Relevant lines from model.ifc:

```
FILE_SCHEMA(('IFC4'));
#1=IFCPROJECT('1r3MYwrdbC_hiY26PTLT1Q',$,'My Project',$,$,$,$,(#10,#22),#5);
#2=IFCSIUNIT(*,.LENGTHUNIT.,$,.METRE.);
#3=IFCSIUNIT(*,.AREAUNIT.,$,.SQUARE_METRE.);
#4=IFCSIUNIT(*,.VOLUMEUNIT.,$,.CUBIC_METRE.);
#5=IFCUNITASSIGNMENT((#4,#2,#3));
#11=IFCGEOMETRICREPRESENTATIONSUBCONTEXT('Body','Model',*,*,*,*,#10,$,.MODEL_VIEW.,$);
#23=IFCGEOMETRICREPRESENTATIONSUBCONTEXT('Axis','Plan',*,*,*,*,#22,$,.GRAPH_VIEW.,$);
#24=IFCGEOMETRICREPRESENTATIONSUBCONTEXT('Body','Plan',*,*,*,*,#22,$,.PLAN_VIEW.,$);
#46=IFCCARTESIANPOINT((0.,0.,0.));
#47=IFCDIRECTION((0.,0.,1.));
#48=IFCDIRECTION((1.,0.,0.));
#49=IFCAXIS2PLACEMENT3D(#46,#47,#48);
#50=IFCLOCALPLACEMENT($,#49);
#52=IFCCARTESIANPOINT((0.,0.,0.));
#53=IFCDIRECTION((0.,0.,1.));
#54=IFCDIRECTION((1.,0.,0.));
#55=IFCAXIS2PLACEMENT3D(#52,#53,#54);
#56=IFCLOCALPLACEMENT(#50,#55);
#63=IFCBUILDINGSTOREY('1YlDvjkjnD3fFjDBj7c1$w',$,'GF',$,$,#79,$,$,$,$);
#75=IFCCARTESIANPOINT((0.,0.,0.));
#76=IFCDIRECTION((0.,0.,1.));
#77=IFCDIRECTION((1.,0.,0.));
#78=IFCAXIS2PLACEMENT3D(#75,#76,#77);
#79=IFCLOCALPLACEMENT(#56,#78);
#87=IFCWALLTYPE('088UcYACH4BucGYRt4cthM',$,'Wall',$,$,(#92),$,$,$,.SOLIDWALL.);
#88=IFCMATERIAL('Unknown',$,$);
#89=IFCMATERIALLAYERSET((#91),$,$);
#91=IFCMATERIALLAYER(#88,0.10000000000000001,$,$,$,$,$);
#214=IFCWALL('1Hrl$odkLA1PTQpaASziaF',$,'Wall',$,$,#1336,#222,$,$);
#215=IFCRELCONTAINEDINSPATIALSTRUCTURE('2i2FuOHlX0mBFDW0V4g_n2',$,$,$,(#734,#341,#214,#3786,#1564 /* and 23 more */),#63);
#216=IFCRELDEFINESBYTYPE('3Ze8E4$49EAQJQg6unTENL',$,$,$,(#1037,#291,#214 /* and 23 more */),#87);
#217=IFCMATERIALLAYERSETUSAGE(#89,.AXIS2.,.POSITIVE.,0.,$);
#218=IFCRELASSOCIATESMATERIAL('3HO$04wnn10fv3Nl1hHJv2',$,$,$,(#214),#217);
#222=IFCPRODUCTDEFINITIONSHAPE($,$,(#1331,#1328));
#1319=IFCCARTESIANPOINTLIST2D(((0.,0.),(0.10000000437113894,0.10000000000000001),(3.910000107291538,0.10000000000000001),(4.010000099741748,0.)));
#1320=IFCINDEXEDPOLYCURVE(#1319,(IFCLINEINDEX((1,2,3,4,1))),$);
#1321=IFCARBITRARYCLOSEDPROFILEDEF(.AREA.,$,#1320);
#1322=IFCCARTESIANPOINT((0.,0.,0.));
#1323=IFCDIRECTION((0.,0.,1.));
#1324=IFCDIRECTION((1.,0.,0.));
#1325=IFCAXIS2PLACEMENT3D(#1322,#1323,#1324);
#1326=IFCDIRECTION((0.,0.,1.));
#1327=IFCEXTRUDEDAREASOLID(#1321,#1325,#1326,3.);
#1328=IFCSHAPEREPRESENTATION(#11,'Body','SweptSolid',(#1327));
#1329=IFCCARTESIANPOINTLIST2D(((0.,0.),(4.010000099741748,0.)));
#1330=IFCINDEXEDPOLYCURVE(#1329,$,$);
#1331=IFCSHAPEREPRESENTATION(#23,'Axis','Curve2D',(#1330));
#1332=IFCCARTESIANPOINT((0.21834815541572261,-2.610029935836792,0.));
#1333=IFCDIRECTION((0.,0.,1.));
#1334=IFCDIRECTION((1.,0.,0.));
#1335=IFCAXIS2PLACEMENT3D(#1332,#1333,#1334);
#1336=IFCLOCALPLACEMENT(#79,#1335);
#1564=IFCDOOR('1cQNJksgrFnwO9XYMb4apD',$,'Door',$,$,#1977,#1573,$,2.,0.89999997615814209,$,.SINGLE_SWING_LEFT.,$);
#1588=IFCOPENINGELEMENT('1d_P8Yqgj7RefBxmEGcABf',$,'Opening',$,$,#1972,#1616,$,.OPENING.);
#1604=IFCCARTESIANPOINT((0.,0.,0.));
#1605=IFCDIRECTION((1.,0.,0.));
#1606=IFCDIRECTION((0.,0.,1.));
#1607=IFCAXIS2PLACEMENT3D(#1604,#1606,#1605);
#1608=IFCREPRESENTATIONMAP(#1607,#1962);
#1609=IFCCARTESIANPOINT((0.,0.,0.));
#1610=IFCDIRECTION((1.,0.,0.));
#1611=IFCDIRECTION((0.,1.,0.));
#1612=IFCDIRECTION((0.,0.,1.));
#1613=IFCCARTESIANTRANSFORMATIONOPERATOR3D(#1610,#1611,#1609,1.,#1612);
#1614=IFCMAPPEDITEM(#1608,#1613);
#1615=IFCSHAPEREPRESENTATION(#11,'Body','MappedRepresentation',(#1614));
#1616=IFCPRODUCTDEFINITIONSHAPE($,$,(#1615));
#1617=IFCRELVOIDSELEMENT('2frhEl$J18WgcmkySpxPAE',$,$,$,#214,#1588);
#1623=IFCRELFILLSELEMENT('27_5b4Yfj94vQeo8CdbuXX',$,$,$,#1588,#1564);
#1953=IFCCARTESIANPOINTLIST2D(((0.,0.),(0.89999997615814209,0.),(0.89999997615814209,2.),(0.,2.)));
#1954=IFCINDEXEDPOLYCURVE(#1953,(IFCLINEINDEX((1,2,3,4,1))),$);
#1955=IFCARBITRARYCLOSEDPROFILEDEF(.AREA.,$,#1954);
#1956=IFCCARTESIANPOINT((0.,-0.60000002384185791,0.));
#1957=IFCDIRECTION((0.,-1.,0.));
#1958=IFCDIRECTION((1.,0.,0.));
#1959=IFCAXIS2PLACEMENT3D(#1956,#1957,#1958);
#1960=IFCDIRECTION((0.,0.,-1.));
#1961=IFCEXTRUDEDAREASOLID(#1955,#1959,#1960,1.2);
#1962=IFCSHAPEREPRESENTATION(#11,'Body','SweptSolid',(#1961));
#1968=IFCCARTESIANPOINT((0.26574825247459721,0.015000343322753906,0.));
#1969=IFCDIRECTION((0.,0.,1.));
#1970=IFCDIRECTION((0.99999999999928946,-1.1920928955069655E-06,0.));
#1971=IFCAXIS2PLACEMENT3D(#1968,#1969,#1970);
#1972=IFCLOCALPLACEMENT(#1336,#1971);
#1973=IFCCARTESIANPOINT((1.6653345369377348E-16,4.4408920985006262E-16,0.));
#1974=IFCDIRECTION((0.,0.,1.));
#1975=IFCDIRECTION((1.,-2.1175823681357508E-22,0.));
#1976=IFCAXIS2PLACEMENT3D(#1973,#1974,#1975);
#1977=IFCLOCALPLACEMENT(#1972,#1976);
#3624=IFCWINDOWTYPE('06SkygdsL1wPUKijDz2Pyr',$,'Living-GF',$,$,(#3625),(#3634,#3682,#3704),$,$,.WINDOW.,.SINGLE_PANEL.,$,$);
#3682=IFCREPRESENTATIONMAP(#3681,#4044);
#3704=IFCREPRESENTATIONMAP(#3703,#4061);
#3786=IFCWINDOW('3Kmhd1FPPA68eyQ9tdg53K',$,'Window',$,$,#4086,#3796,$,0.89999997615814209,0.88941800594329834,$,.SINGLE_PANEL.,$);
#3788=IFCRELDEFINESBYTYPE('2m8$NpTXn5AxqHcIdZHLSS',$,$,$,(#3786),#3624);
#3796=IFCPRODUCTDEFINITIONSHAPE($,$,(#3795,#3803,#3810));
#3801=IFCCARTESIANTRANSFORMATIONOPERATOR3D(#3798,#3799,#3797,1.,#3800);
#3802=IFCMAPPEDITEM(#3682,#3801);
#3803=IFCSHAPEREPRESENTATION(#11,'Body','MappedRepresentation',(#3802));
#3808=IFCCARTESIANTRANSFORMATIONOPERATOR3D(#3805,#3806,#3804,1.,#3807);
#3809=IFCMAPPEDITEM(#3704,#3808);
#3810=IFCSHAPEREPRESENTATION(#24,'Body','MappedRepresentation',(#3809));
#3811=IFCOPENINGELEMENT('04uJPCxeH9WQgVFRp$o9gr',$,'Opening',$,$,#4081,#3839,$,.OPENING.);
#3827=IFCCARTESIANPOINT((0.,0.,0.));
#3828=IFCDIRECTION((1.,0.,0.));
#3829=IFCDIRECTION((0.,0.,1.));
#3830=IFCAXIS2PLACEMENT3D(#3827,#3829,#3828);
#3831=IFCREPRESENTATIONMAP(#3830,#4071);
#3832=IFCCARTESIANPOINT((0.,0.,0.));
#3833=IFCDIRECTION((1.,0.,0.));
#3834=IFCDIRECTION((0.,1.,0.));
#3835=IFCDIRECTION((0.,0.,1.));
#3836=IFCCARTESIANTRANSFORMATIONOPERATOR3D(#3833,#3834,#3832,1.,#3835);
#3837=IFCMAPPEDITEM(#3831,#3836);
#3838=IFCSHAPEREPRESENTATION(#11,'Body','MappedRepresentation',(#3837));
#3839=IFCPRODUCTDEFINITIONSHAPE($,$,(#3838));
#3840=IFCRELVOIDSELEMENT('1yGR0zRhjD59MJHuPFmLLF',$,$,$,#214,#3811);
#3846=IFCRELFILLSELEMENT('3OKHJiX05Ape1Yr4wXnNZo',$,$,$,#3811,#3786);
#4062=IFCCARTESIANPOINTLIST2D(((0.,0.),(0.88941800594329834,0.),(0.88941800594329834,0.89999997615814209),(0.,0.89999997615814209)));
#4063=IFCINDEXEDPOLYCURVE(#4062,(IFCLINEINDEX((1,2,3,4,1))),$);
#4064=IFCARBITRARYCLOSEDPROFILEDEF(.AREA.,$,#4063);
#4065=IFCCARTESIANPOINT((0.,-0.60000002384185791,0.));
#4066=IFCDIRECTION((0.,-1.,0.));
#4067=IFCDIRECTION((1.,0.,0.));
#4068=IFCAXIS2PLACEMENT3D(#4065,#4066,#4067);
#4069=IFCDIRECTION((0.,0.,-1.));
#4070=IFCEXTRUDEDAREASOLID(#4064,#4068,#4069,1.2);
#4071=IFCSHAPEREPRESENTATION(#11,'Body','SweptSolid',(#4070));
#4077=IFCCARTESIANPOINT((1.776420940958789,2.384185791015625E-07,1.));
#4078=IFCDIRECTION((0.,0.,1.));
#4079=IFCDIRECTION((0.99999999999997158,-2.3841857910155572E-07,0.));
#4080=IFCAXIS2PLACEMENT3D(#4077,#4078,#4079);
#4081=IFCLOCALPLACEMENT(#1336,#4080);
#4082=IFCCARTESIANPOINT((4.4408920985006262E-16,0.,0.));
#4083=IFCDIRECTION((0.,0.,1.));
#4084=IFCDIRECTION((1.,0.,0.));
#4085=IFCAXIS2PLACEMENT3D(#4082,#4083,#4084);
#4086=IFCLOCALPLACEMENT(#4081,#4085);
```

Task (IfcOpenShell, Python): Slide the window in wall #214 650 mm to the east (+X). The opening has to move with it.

```python
import ifcopenshell
import ifcopenshell.api.geometry
import ifcopenshell.util.placement
import ifcopenshell.util.unit

model = ifcopenshell.open("model.ifc")
unit_scale = ifcopenshell.util.unit.calculate_unit_scale(model)

window = model.by_guid("3Kmhd1FPPA68eyQ9tdg53K")
opening = window.FillsVoids[0].RelatingOpeningElement
wall = opening.VoidsElements[0].RelatingBuildingElement

wall_matrix = ifcopenshell.util.placement.get_local_placement(wall.ObjectPlacement)
shift = wall_matrix[:3, 0] * 0.65 / unit_scale
before = ifcopenshell.util.placement.get_local_placement(window.ObjectPlacement)[:3, 3].copy()

# The window is placed relative to its opening, so it follows when the opening moves.
matrix = ifcopenshell.util.placement.get_local_placement(opening.ObjectPlacement)
matrix[:3, 3] += shift
ifcopenshell.api.geometry.edit_object_placement(
    model, product=opening, matrix=matrix, is_si=False, should_transform_children=True
)

after = ifcopenshell.util.placement.get_local_placement(window.ObjectPlacement)[:3, 3]
print("window moved by", (after - before).round(3) + 0.0)

model.write("model_updated.ifc")
```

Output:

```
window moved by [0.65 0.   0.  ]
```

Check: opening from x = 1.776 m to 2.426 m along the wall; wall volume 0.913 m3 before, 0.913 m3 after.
